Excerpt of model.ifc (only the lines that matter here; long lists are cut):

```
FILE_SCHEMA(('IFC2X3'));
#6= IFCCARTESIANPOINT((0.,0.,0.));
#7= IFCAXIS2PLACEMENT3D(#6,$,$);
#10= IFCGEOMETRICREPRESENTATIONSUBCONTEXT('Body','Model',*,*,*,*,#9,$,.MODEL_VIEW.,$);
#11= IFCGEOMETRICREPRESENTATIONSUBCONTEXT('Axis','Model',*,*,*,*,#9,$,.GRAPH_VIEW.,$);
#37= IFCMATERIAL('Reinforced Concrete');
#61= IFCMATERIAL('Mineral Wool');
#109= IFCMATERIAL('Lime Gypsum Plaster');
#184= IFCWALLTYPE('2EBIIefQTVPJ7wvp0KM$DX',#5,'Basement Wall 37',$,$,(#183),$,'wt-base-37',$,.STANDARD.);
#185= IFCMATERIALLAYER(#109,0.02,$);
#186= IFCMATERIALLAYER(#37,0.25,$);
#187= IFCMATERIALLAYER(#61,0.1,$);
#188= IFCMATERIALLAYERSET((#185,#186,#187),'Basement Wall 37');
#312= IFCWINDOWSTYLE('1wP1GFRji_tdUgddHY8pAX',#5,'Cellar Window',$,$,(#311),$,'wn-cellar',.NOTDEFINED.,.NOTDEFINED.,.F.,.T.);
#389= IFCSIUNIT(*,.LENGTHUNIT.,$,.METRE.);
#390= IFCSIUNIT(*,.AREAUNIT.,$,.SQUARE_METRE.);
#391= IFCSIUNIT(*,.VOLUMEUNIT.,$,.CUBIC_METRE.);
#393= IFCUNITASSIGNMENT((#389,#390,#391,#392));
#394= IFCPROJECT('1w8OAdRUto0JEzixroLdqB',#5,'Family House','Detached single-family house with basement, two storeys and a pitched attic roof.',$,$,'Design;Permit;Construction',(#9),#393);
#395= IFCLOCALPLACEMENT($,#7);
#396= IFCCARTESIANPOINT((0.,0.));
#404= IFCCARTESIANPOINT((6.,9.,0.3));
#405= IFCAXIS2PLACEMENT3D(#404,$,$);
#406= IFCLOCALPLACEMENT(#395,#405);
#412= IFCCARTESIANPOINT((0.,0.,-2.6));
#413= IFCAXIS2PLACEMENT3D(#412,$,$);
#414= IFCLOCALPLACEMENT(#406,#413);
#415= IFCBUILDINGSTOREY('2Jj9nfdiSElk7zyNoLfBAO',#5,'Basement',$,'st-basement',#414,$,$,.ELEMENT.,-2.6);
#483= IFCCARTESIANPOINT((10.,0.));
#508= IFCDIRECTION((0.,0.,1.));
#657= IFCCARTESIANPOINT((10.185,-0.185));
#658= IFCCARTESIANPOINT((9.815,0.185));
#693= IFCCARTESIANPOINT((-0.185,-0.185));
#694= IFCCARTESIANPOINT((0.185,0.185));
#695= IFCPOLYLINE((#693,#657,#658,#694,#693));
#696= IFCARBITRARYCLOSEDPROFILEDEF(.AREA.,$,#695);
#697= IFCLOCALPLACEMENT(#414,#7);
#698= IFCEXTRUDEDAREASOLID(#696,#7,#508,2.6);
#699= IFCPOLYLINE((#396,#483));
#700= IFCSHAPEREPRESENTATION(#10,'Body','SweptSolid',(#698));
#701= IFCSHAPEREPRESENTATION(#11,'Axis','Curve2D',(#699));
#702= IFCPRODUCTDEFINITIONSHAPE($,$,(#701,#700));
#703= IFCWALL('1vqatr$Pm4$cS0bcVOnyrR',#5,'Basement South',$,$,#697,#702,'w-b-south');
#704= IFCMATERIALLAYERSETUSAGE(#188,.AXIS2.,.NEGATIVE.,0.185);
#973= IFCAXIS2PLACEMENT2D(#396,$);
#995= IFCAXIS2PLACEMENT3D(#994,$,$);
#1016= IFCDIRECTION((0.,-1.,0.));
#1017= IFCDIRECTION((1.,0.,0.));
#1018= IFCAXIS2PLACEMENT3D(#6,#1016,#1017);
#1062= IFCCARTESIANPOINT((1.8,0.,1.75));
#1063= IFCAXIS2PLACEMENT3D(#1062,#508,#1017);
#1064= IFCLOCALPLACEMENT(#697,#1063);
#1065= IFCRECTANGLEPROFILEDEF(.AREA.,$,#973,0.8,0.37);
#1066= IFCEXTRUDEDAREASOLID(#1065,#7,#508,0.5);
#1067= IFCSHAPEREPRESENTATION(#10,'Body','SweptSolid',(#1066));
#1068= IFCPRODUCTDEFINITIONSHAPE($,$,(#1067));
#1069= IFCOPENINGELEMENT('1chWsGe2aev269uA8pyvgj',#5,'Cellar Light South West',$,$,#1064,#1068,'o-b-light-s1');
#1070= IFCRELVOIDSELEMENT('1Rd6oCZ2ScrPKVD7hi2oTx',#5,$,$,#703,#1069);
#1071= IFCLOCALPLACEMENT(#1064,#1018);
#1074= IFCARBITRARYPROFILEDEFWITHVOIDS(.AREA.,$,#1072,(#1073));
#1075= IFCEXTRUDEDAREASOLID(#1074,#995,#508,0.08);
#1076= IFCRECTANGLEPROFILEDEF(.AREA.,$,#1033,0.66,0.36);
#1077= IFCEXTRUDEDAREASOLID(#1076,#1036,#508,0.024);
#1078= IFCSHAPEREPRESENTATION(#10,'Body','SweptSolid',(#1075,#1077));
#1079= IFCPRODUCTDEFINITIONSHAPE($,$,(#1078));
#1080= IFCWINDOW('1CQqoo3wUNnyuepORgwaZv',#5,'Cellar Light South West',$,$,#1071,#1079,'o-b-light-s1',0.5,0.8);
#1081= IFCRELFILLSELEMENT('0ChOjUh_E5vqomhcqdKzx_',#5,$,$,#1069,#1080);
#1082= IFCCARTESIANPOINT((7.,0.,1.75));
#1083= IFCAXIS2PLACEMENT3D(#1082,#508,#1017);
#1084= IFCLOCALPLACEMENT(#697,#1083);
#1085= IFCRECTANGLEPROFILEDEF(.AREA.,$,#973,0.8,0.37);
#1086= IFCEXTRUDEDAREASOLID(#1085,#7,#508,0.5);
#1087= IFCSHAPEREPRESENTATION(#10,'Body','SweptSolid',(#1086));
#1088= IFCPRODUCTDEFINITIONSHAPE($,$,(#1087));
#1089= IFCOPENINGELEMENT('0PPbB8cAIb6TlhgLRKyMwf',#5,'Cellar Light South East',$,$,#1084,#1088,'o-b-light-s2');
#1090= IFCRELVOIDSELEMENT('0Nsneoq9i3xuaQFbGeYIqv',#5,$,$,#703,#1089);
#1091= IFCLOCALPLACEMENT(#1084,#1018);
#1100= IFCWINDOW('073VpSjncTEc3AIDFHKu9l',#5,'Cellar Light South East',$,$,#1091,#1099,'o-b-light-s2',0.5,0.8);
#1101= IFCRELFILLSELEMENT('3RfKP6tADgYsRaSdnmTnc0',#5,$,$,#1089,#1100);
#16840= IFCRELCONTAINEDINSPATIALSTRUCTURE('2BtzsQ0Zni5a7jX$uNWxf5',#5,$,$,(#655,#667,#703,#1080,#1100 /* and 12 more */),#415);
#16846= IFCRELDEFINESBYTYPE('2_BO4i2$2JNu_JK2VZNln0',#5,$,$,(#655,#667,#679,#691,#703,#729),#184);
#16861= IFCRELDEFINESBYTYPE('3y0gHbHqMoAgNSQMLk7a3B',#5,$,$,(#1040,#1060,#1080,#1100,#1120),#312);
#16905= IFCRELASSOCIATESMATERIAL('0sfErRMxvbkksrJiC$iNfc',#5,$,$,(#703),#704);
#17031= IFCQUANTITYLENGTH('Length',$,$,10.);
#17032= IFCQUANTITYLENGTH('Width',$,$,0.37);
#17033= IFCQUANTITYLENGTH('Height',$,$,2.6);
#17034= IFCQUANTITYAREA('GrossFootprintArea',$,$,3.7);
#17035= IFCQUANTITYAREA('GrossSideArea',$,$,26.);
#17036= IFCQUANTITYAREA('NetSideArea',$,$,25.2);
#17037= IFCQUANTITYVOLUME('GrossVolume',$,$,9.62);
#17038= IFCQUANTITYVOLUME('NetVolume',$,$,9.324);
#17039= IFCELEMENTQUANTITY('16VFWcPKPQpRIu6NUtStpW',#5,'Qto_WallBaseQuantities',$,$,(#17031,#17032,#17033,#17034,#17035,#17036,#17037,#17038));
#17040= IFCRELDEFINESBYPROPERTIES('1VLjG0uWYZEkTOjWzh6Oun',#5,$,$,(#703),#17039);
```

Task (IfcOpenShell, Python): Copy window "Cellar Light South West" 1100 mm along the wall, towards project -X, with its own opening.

```python
import ifcopenshell
import ifcopenshell.api.feature
import ifcopenshell.api.geometry
import ifcopenshell.api.pset
import ifcopenshell.api.root
import ifcopenshell.geom
import ifcopenshell.util.element
import ifcopenshell.util.placement
import ifcopenshell.util.shape
import ifcopenshell.util.unit

model = ifcopenshell.open("model.ifc")
unit_scale = ifcopenshell.util.unit.calculate_unit_scale(model)
area_scale = ifcopenshell.util.unit.calculate_unit_scale(model, "AREAUNIT")
volume_scale = ifcopenshell.util.unit.calculate_unit_scale(model, "VOLUMEUNIT")
settings = ifcopenshell.geom.settings()


def volume(element):
    """Net volume in cubic metres, openings subtracted."""
    shape = ifcopenshell.geom.create_shape(settings, element)
    return ifcopenshell.util.shape.get_volume(shape.geometry)


def reuse_history(source, copy):
    """copy_class also copies each property set's owner history, people and application; keep the originals."""
    for rel in copy.IsDefinedBy:
        if rel.is_a("IfcRelDefinesByProperties") and (history := rel.RelatingPropertyDefinition.OwnerHistory):
            rel.RelatingPropertyDefinition.OwnerHistory = source.OwnerHistory
            ifcopenshell.util.element.remove_deep2(model, history)


window = model.by_guid("1CQqoo3wUNnyuepORgwaZv")
opening = window.FillsVoids[0].RelatingOpeningElement
wall = opening.VoidsElements[0].RelatingBuildingElement
before = volume(wall)
shift = ifcopenshell.util.placement.get_local_placement(wall.ObjectPlacement)[:3, 0] * -1.1 / unit_scale

# copy_class copies the void relationship, type, container and properties, but no geometry.
new_opening = ifcopenshell.api.root.copy_class(model, product=opening)
new_opening.Representation = ifcopenshell.util.element.copy_deep(
    model, opening.Representation, exclude=["IfcGeometricRepresentationContext", "IfcRepresentationMap"]
)
new_opening.Tag = None
new_window = ifcopenshell.api.root.copy_class(model, product=window)
new_window.Representation = ifcopenshell.util.element.copy_deep(
    model, window.Representation, exclude=["IfcGeometricRepresentationContext", "IfcRepresentationMap"]
)
new_window.Tag = None
reuse_history(window, new_window)
fills = ifcopenshell.api.feature.add_filling(model, opening=new_opening, element=new_window)
fills.OwnerHistory = new_window.OwnerHistory  # required in IFC2X3

for old, new in ((opening, new_opening), (window, new_window)):
    matrix = ifcopenshell.util.placement.get_local_placement(old.ObjectPlacement)
    matrix[:3, 3] += shift
    ifcopenshell.api.geometry.edit_object_placement(model, product=new, matrix=matrix, is_si=False)

after = volume(wall)
thickness = 0.37  # wall thickness in metres

# Update the wall's stored quantities.
qto = model.by_id(ifcopenshell.util.element.get_pset(wall, "Qto_WallBaseQuantities", should_inherit=False)["id"])
ifcopenshell.api.pset.edit_qto(model, qto=qto, properties={
    "NetSideArea": after / thickness / area_scale,
    "NetVolume": after / volume_scale,
})

print(f"wall volume {before:.3f} -> {after:.3f} m3")

model.write("model_v2.ifc")
```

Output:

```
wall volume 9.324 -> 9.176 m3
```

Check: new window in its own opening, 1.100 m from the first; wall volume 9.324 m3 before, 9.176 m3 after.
